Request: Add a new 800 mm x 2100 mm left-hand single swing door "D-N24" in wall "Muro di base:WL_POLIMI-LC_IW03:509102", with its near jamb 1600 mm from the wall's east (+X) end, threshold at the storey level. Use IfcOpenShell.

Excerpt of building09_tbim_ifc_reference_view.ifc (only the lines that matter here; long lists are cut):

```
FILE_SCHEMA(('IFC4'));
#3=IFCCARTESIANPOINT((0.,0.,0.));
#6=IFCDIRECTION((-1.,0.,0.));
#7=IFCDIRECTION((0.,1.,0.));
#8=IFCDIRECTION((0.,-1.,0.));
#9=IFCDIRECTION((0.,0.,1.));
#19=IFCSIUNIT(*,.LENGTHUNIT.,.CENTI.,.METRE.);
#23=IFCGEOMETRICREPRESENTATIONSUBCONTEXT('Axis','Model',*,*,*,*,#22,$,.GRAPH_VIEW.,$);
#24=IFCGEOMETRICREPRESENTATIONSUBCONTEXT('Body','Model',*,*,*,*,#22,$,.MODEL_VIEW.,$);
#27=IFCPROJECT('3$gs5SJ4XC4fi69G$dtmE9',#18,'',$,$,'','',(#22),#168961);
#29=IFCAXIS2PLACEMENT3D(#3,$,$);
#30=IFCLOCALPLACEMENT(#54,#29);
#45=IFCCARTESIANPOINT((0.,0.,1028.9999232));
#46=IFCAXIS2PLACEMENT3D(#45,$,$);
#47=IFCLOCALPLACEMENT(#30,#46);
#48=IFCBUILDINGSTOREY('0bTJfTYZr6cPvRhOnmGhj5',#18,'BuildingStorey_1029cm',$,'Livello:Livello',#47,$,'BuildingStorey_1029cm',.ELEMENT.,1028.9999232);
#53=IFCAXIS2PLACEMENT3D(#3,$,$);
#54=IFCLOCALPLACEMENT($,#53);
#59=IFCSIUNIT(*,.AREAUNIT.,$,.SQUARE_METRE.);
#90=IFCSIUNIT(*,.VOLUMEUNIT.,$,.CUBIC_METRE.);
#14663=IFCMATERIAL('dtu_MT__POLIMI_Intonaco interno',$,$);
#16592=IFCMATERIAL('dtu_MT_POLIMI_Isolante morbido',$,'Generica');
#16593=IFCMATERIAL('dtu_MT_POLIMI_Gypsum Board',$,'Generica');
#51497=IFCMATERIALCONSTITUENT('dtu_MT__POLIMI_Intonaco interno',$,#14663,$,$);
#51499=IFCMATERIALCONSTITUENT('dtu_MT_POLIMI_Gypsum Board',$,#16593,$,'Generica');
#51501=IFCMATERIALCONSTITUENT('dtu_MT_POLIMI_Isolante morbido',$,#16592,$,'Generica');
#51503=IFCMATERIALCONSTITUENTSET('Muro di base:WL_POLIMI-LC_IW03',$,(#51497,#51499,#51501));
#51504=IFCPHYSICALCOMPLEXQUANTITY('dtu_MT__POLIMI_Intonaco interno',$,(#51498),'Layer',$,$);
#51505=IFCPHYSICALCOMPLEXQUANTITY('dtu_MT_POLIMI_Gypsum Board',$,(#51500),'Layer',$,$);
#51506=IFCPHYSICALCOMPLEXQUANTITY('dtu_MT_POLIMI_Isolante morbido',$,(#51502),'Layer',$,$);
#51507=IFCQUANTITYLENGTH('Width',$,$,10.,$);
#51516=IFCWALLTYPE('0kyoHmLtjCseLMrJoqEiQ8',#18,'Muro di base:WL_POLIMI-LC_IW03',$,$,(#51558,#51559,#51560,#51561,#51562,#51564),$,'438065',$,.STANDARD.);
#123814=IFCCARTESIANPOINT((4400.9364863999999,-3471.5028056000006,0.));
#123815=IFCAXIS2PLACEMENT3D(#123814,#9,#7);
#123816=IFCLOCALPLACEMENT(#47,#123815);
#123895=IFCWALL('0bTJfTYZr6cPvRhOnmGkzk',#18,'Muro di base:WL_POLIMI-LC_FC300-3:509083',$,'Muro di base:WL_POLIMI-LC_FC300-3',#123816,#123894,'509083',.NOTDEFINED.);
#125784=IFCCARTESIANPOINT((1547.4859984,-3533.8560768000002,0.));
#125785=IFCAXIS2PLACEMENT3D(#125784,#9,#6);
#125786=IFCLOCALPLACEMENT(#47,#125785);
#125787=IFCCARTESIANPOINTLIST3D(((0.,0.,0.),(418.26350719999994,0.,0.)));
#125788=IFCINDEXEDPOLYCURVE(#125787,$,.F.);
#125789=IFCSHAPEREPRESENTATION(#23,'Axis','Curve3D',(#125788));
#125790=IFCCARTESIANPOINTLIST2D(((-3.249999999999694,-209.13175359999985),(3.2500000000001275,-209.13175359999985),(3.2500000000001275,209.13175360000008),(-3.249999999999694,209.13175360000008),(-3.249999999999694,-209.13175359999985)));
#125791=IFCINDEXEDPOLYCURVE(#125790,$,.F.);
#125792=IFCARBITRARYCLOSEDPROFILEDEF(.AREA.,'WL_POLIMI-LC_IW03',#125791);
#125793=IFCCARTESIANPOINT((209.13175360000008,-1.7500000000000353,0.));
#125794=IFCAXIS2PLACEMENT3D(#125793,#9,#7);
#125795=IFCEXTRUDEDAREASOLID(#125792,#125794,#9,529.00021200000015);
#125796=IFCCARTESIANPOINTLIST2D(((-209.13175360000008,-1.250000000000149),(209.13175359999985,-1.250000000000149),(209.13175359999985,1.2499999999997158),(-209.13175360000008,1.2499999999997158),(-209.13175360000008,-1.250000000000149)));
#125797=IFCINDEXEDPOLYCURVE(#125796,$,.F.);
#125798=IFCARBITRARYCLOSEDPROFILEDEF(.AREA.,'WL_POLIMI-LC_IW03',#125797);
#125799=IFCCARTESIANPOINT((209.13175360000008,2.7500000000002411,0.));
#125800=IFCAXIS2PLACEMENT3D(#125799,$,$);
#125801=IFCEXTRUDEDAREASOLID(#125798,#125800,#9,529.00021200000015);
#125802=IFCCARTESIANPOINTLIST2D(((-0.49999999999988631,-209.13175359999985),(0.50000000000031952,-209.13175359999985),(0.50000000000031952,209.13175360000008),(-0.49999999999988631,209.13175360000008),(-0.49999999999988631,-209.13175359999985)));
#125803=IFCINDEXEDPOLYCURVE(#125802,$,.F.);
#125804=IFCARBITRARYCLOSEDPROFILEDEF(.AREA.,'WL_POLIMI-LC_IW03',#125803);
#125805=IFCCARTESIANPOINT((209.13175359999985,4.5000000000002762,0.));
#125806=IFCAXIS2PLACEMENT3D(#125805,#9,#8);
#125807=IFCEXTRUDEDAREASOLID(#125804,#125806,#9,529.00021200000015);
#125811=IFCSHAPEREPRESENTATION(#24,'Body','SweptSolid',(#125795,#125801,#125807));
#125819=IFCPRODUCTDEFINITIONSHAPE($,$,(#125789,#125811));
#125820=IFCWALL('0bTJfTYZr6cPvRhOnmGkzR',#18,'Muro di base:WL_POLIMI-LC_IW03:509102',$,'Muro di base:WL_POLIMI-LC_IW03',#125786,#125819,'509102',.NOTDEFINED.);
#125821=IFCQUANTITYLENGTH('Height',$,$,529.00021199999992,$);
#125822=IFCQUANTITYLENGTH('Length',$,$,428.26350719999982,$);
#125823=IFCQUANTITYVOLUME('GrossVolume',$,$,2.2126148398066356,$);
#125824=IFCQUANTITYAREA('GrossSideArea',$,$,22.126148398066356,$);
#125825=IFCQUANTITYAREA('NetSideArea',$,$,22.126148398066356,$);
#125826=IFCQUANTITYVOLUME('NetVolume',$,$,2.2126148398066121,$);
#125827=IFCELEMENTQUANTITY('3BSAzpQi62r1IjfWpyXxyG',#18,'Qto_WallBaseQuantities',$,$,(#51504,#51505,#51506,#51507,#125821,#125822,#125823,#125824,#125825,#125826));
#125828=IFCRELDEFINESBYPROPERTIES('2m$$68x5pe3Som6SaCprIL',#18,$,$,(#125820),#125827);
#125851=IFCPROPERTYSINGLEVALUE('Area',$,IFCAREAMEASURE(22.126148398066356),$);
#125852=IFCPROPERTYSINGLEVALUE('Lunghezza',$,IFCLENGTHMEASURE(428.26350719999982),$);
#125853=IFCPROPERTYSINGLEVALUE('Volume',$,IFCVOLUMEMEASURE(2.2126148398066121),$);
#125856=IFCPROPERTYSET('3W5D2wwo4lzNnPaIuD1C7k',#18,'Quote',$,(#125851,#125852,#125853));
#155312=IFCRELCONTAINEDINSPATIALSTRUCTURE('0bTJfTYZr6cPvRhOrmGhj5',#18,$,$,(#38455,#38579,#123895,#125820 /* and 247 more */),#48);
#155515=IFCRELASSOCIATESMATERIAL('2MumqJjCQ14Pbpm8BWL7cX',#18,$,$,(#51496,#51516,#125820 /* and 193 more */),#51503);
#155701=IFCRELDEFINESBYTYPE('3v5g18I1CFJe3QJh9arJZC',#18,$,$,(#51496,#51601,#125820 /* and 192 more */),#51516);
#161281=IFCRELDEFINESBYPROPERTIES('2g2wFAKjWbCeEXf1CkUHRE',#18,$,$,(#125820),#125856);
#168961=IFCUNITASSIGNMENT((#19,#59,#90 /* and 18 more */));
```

```python
import numpy as np
import ifcopenshell
import ifcopenshell.api.feature
import ifcopenshell.api.geometry
import ifcopenshell.api.pset
import ifcopenshell.api.root
import ifcopenshell.api.spatial
import ifcopenshell.geom
import ifcopenshell.util.element
import ifcopenshell.util.placement
import ifcopenshell.util.representation
import ifcopenshell.util.shape
import ifcopenshell.util.unit

model = ifcopenshell.open("building09_tbim_ifc_reference_view.ifc")
unit_scale = ifcopenshell.util.unit.calculate_unit_scale(model)
area_scale = ifcopenshell.util.unit.calculate_unit_scale(model, "AREAUNIT")
volume_scale = ifcopenshell.util.unit.calculate_unit_scale(model, "VOLUMEUNIT")
settings = ifcopenshell.geom.settings()


def volume(element):
    """Net volume in cubic metres, openings subtracted."""
    shape = ifcopenshell.geom.create_shape(settings, element)
    return ifcopenshell.util.shape.get_volume(shape.geometry)


wall = model.by_guid("0bTJfTYZr6cPvRhOnmGkzR")
storey = ifcopenshell.util.element.get_container(wall, ifc_class="IfcBuildingStorey")
context = ifcopenshell.util.representation.get_context(model, "Model", "Body", "MODEL_VIEW")
before = volume(wall)

width, height, from_end, sill = 0.8, 2.1, 1.6, 0.0  # metres

# The wall runs along its own X axis, and the end named is its -X end.
wall_shape = ifcopenshell.geom.create_shape(settings, wall)
x, y, z = ifcopenshell.util.shape.get_vertices(wall_shape.geometry).T
start = x.min() + from_end
face, thickness = float(y.min()), float(y.max() - y.min())
wall_matrix = ifcopenshell.util.placement.get_local_placement(wall.ObjectPlacement)
level = ifcopenshell.util.placement.get_local_placement(storey.ObjectPlacement)[2, 3]


def in_wall(x, y):
    """Placement at x, y metres in the wall's axes, at sill height."""
    matrix = wall_matrix.copy()
    matrix[:, 3] = wall_matrix @ np.array([x / unit_scale, y / unit_scale, 0.0, 1.0])
    matrix[2, 3] = level + sill / unit_scale
    return matrix


# Opening: a box that overshoots both wall faces by 50 mm.
opening = ifcopenshell.api.root.create_entity(model, ifc_class="IfcOpeningElement", predefined_type="OPENING")
box = ifcopenshell.api.geometry.add_wall_representation(
    model, context=context, length=width, height=height, thickness=thickness + 0.1
)
ifcopenshell.api.geometry.assign_representation(model, product=opening, representation=box)
ifcopenshell.api.geometry.edit_object_placement(model, product=opening, matrix=in_wall(start, face - 0.05), is_si=False)
ifcopenshell.api.feature.add_feature(model, feature=opening, element=wall)

door = ifcopenshell.api.root.create_entity(model, ifc_class="IfcDoor", name="D-N24", predefined_type="DOOR")
door.OverallWidth, door.OverallHeight = width / unit_scale, height / unit_scale
door.OperationType = "SINGLE_SWING_LEFT"
body = ifcopenshell.api.geometry.add_door_representation(
    model,
    context=context,
    overall_width=door.OverallWidth,
    overall_height=door.OverallHeight,
    operation_type="SINGLE_SWING_LEFT",
    lining_properties={"LiningDepth": thickness / unit_scale, "ThresholdDepth": thickness / unit_scale},
)
ifcopenshell.api.geometry.assign_representation(model, product=door, representation=body)
ifcopenshell.api.spatial.assign_container(model, products=[door], relating_structure=storey)
ifcopenshell.api.feature.add_filling(model, opening=opening, element=door)

# The lining spans the wall, so the door starts at the wall face.
ifcopenshell.api.geometry.edit_object_placement(model, product=door, matrix=in_wall(start, face), is_si=False)

after = volume(wall)

# Update the wall's stored quantities.
qto = model.by_id(ifcopenshell.util.element.get_pset(wall, "Qto_WallBaseQuantities", should_inherit=False)["id"])
ifcopenshell.api.pset.edit_qto(model, qto=qto, properties={
    "NetSideArea": after / thickness / area_scale,
    "NetVolume": after / volume_scale,
})
pset = model.by_id(ifcopenshell.util.element.get_pset(wall, "Quote", should_inherit=False)["id"])
ifcopenshell.api.pset.edit_pset(model, pset=pset, properties={
    "Area": model.create_entity("IfcAreaMeasure", after / thickness / area_scale),
    "Volume": model.create_entity("IfcVolumeMeasure", after / volume_scale),
})

print(f"wall volume {before:.3f} -> {after:.3f} m3")

model.write("building09_tbim_ifc_reference_view_v2.ifc")
```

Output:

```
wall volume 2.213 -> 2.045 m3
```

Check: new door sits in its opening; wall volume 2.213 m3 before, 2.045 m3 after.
